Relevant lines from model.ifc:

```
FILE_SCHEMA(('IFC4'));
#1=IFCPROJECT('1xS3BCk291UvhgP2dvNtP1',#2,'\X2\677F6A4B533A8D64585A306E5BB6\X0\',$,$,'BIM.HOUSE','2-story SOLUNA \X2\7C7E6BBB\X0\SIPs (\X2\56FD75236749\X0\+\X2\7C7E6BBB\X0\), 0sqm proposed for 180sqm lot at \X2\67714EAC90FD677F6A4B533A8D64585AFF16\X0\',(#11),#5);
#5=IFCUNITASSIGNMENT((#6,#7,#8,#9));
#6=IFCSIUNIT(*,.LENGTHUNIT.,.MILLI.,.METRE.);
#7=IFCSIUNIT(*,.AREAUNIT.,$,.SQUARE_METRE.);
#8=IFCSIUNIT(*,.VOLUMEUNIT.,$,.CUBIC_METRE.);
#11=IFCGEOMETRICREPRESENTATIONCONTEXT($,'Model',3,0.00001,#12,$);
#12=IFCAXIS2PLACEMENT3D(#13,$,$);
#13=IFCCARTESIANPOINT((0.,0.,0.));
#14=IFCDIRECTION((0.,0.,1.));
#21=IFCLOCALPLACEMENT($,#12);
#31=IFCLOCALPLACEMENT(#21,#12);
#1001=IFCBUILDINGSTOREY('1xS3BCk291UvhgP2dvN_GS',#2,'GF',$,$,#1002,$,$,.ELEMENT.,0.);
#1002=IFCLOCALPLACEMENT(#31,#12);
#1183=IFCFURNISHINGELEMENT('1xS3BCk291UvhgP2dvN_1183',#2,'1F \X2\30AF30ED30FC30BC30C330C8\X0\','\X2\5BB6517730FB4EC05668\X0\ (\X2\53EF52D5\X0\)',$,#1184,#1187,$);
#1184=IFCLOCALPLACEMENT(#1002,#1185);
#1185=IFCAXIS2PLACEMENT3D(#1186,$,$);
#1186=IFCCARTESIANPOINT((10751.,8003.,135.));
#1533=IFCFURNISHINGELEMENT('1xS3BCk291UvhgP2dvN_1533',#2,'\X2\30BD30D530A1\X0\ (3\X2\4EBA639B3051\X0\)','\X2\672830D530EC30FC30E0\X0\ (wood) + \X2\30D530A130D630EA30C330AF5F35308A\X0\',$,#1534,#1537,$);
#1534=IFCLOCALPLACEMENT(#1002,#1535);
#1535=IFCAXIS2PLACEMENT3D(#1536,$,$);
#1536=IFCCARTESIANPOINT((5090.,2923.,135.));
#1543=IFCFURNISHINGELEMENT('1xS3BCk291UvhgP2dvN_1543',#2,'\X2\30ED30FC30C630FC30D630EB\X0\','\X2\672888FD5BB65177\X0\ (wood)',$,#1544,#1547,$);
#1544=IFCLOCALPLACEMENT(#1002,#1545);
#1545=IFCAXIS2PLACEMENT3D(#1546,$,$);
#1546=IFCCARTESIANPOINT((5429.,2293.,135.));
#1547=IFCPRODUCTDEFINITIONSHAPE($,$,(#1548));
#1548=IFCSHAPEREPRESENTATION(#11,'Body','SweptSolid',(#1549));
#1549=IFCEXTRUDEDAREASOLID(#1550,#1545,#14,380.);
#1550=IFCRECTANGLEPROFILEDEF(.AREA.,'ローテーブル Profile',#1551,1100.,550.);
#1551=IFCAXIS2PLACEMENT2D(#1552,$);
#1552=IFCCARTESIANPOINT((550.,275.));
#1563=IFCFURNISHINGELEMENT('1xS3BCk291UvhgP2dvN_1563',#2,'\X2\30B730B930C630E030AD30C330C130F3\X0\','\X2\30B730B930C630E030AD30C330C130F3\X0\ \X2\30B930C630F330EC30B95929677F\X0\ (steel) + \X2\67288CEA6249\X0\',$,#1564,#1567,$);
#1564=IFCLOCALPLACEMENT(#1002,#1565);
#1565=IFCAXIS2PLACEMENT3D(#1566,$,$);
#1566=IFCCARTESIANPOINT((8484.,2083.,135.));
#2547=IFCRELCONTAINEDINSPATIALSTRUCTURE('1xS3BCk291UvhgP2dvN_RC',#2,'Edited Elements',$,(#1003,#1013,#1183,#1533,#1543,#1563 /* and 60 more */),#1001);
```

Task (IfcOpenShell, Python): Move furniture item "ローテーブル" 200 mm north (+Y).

```python
import ifcopenshell
import ifcopenshell.api.geometry
import ifcopenshell.util.placement

model = ifcopenshell.open("model.ifc")

item = model.by_guid("1xS3BCk291UvhgP2dvN_1543")
matrix = ifcopenshell.util.placement.get_local_placement(item.ObjectPlacement)
matrix[1, 3] += 200.0
ifcopenshell.api.geometry.edit_object_placement(model, product=item, matrix=matrix, is_si=False)

print(ifcopenshell.util.placement.get_local_placement(item.ObjectPlacement).round(3) + 0.0)

model.write("model-out.ifc")
```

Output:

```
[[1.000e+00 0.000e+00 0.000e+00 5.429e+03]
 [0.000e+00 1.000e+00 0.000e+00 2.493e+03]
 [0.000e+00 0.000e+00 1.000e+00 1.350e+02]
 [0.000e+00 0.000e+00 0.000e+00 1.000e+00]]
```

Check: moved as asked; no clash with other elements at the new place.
